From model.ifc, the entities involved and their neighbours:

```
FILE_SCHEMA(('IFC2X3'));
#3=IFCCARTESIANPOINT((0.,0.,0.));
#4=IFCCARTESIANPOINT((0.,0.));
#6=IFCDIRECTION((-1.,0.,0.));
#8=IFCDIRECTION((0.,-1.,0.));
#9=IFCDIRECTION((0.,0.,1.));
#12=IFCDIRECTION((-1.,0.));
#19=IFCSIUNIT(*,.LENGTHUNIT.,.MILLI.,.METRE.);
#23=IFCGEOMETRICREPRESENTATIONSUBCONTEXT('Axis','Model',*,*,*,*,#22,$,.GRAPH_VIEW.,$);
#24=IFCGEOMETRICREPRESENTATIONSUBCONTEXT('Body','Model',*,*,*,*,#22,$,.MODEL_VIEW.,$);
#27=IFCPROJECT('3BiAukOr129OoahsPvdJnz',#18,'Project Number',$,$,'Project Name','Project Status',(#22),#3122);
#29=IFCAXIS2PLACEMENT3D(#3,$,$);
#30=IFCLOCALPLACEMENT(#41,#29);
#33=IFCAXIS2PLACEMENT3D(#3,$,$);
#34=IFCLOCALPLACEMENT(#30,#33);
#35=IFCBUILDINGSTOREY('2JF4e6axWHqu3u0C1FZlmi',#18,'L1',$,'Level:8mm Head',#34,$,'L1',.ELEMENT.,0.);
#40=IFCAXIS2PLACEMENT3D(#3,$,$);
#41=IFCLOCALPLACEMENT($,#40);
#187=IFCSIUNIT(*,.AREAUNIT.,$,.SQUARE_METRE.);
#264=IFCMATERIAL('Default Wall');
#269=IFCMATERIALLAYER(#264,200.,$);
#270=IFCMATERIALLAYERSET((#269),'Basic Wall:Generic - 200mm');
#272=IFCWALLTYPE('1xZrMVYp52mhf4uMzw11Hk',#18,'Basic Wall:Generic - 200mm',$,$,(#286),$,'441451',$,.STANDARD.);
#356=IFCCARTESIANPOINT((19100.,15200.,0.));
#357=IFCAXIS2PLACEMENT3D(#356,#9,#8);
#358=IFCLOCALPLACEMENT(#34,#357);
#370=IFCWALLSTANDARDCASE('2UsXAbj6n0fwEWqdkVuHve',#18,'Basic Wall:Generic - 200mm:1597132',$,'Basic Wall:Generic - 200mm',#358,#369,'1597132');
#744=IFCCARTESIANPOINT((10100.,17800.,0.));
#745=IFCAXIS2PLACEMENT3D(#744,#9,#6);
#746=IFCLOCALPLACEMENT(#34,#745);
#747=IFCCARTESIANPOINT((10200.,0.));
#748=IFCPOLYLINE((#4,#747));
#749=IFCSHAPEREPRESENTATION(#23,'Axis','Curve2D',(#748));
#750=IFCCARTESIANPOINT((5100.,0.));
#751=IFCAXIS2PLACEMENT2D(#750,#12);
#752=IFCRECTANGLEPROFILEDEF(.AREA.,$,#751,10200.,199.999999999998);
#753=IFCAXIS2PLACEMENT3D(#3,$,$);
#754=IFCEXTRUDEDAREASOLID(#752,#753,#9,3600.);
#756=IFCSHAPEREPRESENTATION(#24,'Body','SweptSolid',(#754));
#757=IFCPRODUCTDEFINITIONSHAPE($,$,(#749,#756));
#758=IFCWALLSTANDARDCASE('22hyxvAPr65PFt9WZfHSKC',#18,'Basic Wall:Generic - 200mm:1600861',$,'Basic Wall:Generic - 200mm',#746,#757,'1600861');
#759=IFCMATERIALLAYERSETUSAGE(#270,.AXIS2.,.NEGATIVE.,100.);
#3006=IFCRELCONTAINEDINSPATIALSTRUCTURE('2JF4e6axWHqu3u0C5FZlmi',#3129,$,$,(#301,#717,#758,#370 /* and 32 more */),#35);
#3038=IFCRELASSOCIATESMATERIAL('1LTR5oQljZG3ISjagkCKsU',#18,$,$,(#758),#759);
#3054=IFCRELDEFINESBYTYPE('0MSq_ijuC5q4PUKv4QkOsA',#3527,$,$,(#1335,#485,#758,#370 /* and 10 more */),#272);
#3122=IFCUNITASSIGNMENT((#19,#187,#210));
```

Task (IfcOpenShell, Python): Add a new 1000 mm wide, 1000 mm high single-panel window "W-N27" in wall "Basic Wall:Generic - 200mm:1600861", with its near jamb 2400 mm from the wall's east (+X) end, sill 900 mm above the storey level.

```python
import numpy as np
import ifcopenshell
import ifcopenshell.api.feature
import ifcopenshell.api.geometry
import ifcopenshell.api.root
import ifcopenshell.api.spatial
import ifcopenshell.api.type
import ifcopenshell.geom
import ifcopenshell.util.element
import ifcopenshell.util.placement
import ifcopenshell.util.representation
import ifcopenshell.util.shape
import ifcopenshell.util.unit

model = ifcopenshell.open("model.ifc")
unit_scale = ifcopenshell.util.unit.calculate_unit_scale(model)
settings = ifcopenshell.geom.settings()


def volume(element):
    """Net volume in cubic metres, openings subtracted."""
    shape = ifcopenshell.geom.create_shape(settings, element)
    return ifcopenshell.util.shape.get_volume(shape.geometry)


wall = model.by_id(758)
storey = ifcopenshell.util.element.get_container(wall, ifc_class="IfcBuildingStorey")
context = ifcopenshell.util.representation.get_context(model, "Model", "Body", "MODEL_VIEW")
before = volume(wall)

width, height, from_end, sill = 1, 1, 2.4, 0.9  # metres

# The wall runs along its own X axis, and the end named is its -X end.
wall_shape = ifcopenshell.geom.create_shape(settings, wall)
x, y, z = ifcopenshell.util.shape.get_vertices(wall_shape.geometry).T
start = x.min() + from_end
face, thickness = float(y.min()), float(y.max() - y.min())
wall_matrix = ifcopenshell.util.placement.get_local_placement(wall.ObjectPlacement)
level = ifcopenshell.util.placement.get_local_placement(storey.ObjectPlacement)[2, 3]


def in_wall(x, y):
    """Placement at x, y metres in the wall's axes, at sill height."""
    matrix = wall_matrix.copy()
    matrix[:, 3] = wall_matrix @ np.array([x / unit_scale, y / unit_scale, 0.0, 1.0])
    matrix[2, 3] = level + sill / unit_scale
    return matrix


# Opening: a box that overshoots both wall faces by 50 mm.
opening = ifcopenshell.api.root.create_entity(model, ifc_class="IfcOpeningElement")
box = ifcopenshell.api.geometry.add_wall_representation(
    model, context=context, length=width, height=height, thickness=thickness + 0.1
)
ifcopenshell.api.geometry.assign_representation(model, product=opening, representation=box)
ifcopenshell.api.geometry.edit_object_placement(model, product=opening, matrix=in_wall(start, face - 0.05), is_si=False)
ifcopenshell.api.feature.add_feature(model, feature=opening, element=wall)

window = ifcopenshell.api.root.create_entity(model, ifc_class="IfcWindow", name="W-N27")
window.OverallWidth, window.OverallHeight = width / unit_scale, height / unit_scale
body = ifcopenshell.api.geometry.add_window_representation(
    model,
    context=context,
    overall_width=window.OverallWidth,
    overall_height=window.OverallHeight,
    partition_type="SINGLE_PANEL",
)
ifcopenshell.api.geometry.assign_representation(model, product=window, representation=body)
ifcopenshell.api.spatial.assign_container(model, products=[window], relating_structure=storey)
fills = ifcopenshell.api.feature.add_filling(model, opening=opening, element=window)
fills.OwnerHistory = window.OwnerHistory  # required in IFC2X3

# IFC2X3 keeps the operation on the window style.
style = ifcopenshell.api.root.create_entity(model, ifc_class="IfcWindowStyle", name="W-N27")
style.OperationType, style.ConstructionType = "SINGLE_PANEL", "NOTDEFINED"
style.ParameterTakesPrecedence = style.Sizeable = False
ifcopenshell.api.type.assign_type(model, related_objects=[window], relating_type=style)

# Centre the window in the wall's thickness.
ifcopenshell.api.geometry.edit_object_placement(model, product=window, matrix=in_wall(start, face), is_si=False)
window_shape = ifcopenshell.geom.create_shape(settings, window)
depth = ifcopenshell.util.shape.get_vertices(window_shape.geometry)[:, 1]
offset = face + thickness / 2 - (depth.min() + depth.max()) / 2
ifcopenshell.api.geometry.edit_object_placement(model, product=window, matrix=in_wall(start, offset), is_si=False)

after = volume(wall)

print(f"wall volume {before:.3f} -> {after:.3f} m3")

model.write("model_rev.ifc")
```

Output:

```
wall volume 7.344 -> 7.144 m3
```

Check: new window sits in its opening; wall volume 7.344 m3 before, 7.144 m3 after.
